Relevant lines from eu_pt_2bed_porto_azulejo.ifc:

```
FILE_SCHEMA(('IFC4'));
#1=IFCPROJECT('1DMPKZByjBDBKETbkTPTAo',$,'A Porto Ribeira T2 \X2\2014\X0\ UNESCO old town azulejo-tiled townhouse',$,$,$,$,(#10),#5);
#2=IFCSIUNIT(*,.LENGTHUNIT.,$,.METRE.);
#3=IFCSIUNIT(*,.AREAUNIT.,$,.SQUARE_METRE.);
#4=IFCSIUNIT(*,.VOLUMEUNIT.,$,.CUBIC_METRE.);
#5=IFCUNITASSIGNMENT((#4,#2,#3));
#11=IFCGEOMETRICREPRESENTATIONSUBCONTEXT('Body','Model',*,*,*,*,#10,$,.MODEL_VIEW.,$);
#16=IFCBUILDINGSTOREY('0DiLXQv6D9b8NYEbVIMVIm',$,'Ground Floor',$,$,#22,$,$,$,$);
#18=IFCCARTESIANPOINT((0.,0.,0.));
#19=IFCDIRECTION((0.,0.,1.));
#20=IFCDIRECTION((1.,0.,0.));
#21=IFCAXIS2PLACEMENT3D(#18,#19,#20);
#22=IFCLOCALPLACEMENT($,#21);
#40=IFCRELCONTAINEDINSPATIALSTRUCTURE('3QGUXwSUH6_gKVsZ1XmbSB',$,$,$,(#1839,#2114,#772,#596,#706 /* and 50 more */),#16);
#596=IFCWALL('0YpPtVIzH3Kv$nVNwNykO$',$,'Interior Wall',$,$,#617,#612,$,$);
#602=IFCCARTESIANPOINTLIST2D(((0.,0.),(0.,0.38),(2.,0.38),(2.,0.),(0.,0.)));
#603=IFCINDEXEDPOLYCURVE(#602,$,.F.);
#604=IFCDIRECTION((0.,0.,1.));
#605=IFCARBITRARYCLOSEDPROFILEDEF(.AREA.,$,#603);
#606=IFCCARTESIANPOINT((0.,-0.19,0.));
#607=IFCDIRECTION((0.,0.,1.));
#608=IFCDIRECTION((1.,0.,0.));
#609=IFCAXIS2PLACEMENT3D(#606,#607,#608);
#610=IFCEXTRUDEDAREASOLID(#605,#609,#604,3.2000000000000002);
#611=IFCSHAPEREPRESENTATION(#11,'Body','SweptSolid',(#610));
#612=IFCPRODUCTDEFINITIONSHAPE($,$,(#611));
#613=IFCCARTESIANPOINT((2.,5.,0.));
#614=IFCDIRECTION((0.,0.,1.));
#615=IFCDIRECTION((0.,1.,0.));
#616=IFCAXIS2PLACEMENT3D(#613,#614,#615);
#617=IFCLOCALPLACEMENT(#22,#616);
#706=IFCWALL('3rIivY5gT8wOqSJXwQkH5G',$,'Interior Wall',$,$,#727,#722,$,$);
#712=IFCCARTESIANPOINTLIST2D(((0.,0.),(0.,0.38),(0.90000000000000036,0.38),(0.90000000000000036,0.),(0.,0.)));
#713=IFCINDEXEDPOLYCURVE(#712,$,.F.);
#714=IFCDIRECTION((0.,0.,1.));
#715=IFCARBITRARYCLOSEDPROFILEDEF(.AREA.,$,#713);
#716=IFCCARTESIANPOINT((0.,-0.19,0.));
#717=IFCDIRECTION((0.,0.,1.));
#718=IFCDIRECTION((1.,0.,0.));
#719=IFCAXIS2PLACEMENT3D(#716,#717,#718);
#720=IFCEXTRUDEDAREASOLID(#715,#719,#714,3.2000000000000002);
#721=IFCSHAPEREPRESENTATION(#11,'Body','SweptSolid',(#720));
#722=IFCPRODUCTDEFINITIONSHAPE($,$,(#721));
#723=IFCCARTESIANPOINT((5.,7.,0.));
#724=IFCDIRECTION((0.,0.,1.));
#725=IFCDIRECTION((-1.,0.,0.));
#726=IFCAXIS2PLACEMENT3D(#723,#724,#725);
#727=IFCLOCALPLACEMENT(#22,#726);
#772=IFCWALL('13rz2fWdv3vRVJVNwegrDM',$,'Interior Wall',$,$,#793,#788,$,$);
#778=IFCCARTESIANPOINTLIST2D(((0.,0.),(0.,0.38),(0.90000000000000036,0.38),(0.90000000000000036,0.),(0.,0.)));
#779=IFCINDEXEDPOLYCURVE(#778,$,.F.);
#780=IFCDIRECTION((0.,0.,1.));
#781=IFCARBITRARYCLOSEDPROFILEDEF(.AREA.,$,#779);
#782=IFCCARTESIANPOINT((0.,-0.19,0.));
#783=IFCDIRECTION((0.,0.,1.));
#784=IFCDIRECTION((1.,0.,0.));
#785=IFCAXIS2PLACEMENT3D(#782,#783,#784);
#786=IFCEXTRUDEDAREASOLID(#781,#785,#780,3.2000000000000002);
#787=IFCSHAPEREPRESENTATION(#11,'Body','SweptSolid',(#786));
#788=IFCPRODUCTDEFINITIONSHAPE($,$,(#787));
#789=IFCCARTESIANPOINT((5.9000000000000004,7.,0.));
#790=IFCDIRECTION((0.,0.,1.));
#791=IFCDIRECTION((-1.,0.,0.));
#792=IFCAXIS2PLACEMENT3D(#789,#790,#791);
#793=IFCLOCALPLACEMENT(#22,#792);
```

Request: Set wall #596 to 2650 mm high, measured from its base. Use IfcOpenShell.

```python
import ifcopenshell
import ifcopenshell.geom
import ifcopenshell.util.representation
import ifcopenshell.util.shape
import ifcopenshell.util.unit

model = ifcopenshell.open("eu_pt_2bed_porto_azulejo.ifc")
unit_scale = ifcopenshell.util.unit.calculate_unit_scale(model)
settings = ifcopenshell.geom.settings()


def volume(element):
    """Net volume in cubic metres, openings subtracted."""
    shape = ifcopenshell.geom.create_shape(settings, element)
    return ifcopenshell.util.shape.get_volume(shape.geometry)


wall = model.by_id(596)
before = volume(wall)

body = ifcopenshell.util.representation.get_representation(wall, "Model", "Body")
solid = body.Items[0]
old_height = solid.Depth
solid.Depth = 2.65 / unit_scale
after = volume(wall)

print(f"height {old_height:g} -> {solid.Depth:g}, volume {before:.3f} -> {after:.3f} m3")

model.write("eu_pt_2bed_porto_azulejo_v2.ifc")
```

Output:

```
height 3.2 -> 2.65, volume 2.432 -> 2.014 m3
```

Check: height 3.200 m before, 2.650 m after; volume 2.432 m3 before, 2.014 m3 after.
